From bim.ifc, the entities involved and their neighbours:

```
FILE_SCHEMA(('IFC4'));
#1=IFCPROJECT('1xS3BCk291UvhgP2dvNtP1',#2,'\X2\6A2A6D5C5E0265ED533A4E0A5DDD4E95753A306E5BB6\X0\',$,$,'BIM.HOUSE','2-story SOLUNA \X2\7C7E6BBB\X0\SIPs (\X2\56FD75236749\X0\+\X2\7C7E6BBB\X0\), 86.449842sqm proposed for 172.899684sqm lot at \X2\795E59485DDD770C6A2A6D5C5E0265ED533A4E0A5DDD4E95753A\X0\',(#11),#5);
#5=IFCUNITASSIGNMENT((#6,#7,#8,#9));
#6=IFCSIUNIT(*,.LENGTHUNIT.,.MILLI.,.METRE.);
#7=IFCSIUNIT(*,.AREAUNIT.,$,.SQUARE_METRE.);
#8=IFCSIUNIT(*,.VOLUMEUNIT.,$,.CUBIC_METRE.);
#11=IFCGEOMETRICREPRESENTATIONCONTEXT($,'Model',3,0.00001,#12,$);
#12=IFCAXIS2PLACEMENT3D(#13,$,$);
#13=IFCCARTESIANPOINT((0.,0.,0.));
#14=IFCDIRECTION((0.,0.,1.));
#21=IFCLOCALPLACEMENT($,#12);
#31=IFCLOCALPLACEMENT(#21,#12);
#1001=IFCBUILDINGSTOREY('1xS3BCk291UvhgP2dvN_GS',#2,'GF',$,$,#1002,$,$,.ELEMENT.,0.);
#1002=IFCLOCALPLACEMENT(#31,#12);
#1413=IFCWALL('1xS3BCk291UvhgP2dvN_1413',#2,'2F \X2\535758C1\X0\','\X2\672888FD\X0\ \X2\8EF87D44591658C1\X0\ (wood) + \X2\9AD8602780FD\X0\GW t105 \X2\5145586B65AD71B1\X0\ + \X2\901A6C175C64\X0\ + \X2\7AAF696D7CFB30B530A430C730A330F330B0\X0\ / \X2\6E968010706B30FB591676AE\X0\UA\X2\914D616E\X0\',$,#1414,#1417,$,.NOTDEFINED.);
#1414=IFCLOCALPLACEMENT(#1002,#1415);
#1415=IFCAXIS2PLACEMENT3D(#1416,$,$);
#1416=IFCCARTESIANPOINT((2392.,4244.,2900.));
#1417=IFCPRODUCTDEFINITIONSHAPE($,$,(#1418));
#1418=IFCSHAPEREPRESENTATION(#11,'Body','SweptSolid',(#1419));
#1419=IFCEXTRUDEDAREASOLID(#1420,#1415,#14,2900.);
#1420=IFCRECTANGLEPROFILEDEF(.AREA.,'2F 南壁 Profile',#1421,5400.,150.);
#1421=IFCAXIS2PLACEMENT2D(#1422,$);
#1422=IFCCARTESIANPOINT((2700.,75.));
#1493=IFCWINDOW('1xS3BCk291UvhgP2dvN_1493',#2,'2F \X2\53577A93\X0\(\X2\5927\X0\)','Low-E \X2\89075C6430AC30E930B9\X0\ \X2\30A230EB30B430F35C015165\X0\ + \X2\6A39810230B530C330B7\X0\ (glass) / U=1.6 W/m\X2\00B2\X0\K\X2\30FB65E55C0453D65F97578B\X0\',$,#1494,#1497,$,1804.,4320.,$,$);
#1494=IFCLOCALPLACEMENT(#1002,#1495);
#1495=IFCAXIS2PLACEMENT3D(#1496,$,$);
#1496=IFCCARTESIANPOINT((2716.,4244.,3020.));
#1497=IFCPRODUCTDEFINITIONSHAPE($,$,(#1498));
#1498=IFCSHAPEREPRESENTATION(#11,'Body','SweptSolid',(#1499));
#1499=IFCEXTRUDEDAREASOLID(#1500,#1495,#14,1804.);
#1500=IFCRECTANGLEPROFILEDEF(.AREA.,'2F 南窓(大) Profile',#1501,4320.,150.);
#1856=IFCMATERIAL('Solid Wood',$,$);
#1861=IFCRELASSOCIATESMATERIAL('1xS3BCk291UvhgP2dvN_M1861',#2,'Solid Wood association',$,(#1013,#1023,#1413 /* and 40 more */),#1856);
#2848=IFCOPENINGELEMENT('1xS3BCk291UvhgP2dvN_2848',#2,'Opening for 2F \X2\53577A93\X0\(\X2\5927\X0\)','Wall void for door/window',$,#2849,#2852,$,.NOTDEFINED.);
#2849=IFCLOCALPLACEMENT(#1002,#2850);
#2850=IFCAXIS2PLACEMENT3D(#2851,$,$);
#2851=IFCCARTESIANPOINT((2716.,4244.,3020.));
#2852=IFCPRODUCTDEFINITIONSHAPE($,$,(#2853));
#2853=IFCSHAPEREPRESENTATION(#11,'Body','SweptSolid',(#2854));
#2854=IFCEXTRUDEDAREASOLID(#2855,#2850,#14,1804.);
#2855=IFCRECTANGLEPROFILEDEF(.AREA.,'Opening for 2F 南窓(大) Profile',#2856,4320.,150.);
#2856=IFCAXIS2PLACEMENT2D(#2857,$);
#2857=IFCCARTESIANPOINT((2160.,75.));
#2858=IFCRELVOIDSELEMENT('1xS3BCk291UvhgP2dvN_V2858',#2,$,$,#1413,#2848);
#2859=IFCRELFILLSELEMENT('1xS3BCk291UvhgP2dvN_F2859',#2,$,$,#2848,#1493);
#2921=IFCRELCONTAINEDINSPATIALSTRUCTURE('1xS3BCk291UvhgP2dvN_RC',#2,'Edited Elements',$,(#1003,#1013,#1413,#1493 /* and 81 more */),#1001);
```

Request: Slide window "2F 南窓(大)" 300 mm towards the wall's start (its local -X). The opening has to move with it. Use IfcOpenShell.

```python
import ifcopenshell
import ifcopenshell.api.geometry
import ifcopenshell.util.placement

model = ifcopenshell.open("bim.ifc")

window = model.by_id(1493)
opening = window.FillsVoids[0].RelatingOpeningElement
wall = opening.VoidsElements[0].RelatingBuildingElement

wall_matrix = ifcopenshell.util.placement.get_local_placement(wall.ObjectPlacement)
shift = wall_matrix[:3, 0] * -300.0
before = ifcopenshell.util.placement.get_local_placement(window.ObjectPlacement)[:3, 3].copy()

# The window is not placed relative to its opening, so move both.
for product in (opening, window):
    matrix = ifcopenshell.util.placement.get_local_placement(product.ObjectPlacement)
    matrix[:3, 3] += shift
    ifcopenshell.api.geometry.edit_object_placement(model, product=product, matrix=matrix, is_si=False)

after = ifcopenshell.util.placement.get_local_placement(window.ObjectPlacement)[:3, 3]
print("window moved by", (after - before).round(3) + 0.0)

model.write("bim_edited.ifc")
```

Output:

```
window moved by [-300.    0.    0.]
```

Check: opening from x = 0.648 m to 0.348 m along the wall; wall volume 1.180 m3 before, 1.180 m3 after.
